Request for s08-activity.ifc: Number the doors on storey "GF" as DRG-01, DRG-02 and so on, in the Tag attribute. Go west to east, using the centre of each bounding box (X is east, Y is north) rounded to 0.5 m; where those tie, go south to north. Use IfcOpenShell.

First a look at what the model holds.

```python
import ifcopenshell
import ifcopenshell.util.element
import ifcopenshell.util.placement

model = ifcopenshell.open("s08-activity.ifc")
print(model.schema)
storey = next(s for s in model.by_type("IfcBuildingStorey") if s.Name == "GF")
doors = [e for e in ifcopenshell.util.element.get_decomposition(storey) if e.is_a("IfcDoor")]
for e in sorted(doors, key=lambda e: e.id()):
    origin = ifcopenshell.util.placement.get_local_placement(e.ObjectPlacement)[:3, 3]
    print(e.id(), e.Tag, e.Name, origin.round(2) + 0.0, sep=" | ")
```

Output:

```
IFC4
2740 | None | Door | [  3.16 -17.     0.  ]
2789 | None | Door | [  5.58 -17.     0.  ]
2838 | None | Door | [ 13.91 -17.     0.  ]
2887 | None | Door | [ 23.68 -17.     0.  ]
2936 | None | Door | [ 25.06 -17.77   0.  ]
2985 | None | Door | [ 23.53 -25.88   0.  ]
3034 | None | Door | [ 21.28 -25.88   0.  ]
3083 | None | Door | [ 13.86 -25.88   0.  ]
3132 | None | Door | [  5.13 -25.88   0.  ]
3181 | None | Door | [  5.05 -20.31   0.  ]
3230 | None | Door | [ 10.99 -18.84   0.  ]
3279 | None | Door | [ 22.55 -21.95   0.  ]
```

```python
import ifcopenshell
import ifcopenshell.geom
import ifcopenshell.util.element
import ifcopenshell.util.shape

model = ifcopenshell.open("s08-activity.ifc")
settings = ifcopenshell.geom.settings()
settings.set("use-world-coords", True)


def centre(element):
    shape = ifcopenshell.geom.create_shape(settings, element)
    return ifcopenshell.util.shape.get_bbox_centroid(shape.geometry)


storey = next(s for s in model.by_type("IfcBuildingStorey") if s.Name == "GF")
doors = [e for e in ifcopenshell.util.element.get_decomposition(storey) if e.is_a("IfcDoor")]

# Insertion points can sit at a corner or the storey origin, so sort by the geometry (in metres).
centres = {e: centre(e) for e in doors}
doors.sort(key=lambda e: (round(centres[e][0] / 0.5), centres[e][1]))

for i, e in enumerate(doors, start=1):
    number = f"DRG-{i:02d}"
    e.Tag = number
    print(e.id(), number)

model.write("s08-activity_edited.ifc")
```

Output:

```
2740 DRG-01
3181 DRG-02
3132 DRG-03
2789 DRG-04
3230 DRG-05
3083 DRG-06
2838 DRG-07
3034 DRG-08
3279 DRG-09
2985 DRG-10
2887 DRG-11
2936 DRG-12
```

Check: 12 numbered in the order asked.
